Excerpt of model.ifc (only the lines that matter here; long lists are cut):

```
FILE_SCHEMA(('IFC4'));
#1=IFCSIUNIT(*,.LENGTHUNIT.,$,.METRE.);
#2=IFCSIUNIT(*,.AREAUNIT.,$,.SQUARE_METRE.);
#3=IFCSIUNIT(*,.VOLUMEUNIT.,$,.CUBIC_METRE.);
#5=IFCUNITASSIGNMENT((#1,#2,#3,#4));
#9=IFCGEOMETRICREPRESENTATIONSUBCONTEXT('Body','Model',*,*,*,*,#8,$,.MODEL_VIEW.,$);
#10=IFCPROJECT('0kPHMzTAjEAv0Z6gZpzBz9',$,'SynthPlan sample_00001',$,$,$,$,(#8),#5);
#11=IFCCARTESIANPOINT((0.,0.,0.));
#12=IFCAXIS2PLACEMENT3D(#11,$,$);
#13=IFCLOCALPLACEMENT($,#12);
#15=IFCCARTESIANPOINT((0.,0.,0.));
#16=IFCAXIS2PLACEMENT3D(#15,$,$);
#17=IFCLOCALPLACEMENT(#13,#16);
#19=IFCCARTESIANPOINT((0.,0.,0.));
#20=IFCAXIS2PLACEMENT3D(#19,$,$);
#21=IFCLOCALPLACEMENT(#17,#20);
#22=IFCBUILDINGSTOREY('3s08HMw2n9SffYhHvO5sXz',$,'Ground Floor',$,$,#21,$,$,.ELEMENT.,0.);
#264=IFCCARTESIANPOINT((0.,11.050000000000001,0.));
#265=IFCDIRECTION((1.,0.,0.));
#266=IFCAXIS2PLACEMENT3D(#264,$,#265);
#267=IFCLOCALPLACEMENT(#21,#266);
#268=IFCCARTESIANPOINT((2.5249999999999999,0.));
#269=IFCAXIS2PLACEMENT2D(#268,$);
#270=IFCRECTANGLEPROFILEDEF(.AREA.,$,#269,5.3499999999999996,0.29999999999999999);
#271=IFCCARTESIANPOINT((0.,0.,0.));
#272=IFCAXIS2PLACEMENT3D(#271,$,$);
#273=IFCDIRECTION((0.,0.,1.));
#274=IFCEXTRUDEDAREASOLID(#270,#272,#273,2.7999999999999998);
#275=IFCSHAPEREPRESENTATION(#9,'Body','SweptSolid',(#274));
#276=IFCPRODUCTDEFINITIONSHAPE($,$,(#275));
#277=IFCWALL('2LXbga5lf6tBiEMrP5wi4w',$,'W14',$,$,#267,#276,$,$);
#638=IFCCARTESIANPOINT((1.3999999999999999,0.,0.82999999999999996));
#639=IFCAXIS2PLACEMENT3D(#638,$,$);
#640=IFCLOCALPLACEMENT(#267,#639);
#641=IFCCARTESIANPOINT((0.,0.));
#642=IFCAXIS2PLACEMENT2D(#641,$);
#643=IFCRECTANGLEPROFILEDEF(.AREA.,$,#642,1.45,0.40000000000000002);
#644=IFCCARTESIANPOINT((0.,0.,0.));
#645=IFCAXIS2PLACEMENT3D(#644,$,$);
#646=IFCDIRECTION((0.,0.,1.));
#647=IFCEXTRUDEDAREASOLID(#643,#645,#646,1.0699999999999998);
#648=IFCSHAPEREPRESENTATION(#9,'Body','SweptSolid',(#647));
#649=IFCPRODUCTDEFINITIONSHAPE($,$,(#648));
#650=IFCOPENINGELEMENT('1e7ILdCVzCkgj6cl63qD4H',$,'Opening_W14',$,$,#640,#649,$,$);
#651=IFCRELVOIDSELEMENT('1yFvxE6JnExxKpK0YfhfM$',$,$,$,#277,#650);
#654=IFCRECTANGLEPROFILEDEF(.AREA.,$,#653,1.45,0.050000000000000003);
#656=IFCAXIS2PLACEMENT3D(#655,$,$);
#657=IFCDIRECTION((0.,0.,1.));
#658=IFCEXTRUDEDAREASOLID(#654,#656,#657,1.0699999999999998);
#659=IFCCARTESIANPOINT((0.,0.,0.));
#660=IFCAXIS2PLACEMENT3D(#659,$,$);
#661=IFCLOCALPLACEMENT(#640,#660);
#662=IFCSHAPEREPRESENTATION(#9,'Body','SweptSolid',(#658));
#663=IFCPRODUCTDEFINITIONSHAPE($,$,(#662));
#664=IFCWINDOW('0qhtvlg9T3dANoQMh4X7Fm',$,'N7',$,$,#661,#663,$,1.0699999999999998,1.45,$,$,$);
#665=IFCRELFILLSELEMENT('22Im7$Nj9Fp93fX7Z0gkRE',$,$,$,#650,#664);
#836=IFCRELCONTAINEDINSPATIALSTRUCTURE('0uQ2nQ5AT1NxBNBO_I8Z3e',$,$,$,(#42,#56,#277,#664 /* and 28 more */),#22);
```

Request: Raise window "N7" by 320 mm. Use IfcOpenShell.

```python
import numpy as np
import ifcopenshell
import ifcopenshell.api.geometry
import ifcopenshell.util.placement
import ifcopenshell.util.unit

model = ifcopenshell.open("model.ifc")
unit_scale = ifcopenshell.util.unit.calculate_unit_scale(model)

window = model.by_guid("0qhtvlg9T3dANoQMh4X7Fm")
opening = window.FillsVoids[0].RelatingOpeningElement
dz = 0.32

shift = np.array([0.0, 0.0, dz])
# The window is placed relative to its opening, so it follows when the opening moves.
matrix = ifcopenshell.util.placement.get_local_placement(opening.ObjectPlacement)
matrix[:3, 3] += shift
ifcopenshell.api.geometry.edit_object_placement(
    model, product=opening, matrix=matrix, is_si=False, should_transform_children=True
)

print(f"moved by {dz * unit_scale:+.3f} m")

model.write("model_v2.ifc")
```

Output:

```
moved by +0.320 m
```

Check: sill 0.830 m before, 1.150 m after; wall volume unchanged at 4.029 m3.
